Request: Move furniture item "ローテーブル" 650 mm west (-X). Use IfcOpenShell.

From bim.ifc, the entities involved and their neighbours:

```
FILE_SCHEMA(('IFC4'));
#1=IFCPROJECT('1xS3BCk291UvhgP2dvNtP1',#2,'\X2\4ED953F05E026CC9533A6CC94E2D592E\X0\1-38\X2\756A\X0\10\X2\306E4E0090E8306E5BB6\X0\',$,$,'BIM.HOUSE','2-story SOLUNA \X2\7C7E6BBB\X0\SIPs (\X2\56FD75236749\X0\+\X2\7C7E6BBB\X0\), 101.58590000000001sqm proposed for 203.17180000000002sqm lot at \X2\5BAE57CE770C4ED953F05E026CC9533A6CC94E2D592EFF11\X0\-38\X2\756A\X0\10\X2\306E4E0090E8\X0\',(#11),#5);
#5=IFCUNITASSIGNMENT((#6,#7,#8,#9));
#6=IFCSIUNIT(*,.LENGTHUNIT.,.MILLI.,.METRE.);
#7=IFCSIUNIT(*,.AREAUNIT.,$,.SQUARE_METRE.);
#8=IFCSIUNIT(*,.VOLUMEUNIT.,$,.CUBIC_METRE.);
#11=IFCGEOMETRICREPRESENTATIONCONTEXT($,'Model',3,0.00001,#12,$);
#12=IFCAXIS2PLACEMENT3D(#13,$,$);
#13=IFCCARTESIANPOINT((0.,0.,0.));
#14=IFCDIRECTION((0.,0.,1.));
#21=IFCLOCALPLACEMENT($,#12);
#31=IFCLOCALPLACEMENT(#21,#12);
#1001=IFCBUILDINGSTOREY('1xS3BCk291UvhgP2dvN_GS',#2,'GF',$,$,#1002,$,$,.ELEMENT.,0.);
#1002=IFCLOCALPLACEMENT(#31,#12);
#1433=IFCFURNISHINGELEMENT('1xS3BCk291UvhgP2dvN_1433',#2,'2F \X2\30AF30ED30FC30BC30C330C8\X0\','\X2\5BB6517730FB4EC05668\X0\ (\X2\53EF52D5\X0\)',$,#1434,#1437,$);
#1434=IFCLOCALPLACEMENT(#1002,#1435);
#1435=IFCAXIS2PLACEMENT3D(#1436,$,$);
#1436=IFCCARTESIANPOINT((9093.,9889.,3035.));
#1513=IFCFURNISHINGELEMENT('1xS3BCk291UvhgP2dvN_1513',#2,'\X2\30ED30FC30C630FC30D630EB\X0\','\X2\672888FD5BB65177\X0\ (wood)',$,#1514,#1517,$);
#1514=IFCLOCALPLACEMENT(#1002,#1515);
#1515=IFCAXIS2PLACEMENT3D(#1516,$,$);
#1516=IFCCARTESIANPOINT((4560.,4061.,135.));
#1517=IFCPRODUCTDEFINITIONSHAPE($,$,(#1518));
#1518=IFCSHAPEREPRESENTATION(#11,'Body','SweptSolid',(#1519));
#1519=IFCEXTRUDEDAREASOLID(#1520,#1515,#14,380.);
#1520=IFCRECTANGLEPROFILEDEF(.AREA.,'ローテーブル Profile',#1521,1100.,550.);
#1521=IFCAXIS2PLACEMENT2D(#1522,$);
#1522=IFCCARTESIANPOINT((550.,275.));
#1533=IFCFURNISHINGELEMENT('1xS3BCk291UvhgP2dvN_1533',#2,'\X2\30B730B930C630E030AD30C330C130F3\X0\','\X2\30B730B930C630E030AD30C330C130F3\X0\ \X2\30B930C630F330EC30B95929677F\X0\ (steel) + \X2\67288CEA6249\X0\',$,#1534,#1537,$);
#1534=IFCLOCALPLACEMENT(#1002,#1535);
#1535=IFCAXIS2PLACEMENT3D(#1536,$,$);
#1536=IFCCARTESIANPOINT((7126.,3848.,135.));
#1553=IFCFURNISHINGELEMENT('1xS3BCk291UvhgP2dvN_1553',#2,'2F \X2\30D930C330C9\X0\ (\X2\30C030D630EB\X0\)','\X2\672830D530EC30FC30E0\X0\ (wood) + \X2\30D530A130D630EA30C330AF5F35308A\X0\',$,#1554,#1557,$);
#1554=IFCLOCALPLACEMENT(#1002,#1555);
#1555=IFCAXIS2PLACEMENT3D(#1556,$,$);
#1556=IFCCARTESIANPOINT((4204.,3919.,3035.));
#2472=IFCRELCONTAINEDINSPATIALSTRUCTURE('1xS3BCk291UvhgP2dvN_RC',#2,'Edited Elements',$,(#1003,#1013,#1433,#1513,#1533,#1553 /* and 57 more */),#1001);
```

```python
import ifcopenshell
import ifcopenshell.api.geometry
import ifcopenshell.util.placement

model = ifcopenshell.open("bim.ifc")

item = model.by_guid("1xS3BCk291UvhgP2dvN_1513")
matrix = ifcopenshell.util.placement.get_local_placement(item.ObjectPlacement)
matrix[0, 3] -= 650.0
ifcopenshell.api.geometry.edit_object_placement(model, product=item, matrix=matrix, is_si=False)

print(ifcopenshell.util.placement.get_local_placement(item.ObjectPlacement).round(3) + 0.0)

model.write("bim_v2.ifc")
```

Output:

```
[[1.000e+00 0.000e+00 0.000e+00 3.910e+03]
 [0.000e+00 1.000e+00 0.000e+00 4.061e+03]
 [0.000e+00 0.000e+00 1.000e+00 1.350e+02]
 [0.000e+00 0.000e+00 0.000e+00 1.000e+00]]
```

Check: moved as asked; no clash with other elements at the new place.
